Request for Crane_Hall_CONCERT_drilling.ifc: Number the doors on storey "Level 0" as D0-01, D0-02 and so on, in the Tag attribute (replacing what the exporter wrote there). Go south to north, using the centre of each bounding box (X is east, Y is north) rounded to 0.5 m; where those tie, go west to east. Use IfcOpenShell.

First a look at what the model holds.

```python
import ifcopenshell
import ifcopenshell.util.element
import ifcopenshell.util.placement

model = ifcopenshell.open("Crane_Hall_CONCERT_drilling.ifc")
print(model.schema)
storey = next(s for s in model.by_type("IfcBuildingStorey") if s.Name == "Level 0")
doors = [e for e in ifcopenshell.util.element.get_decomposition(storey) if e.is_a("IfcDoor")]
for e in sorted(doors, key=lambda e: e.id()):
    origin = ifcopenshell.util.placement.get_local_placement(e.ObjectPlacement)[:3, 3]
    print(e.id(), e.Tag, e.Name, origin.round(2) + 0.0, sep=" | ")
```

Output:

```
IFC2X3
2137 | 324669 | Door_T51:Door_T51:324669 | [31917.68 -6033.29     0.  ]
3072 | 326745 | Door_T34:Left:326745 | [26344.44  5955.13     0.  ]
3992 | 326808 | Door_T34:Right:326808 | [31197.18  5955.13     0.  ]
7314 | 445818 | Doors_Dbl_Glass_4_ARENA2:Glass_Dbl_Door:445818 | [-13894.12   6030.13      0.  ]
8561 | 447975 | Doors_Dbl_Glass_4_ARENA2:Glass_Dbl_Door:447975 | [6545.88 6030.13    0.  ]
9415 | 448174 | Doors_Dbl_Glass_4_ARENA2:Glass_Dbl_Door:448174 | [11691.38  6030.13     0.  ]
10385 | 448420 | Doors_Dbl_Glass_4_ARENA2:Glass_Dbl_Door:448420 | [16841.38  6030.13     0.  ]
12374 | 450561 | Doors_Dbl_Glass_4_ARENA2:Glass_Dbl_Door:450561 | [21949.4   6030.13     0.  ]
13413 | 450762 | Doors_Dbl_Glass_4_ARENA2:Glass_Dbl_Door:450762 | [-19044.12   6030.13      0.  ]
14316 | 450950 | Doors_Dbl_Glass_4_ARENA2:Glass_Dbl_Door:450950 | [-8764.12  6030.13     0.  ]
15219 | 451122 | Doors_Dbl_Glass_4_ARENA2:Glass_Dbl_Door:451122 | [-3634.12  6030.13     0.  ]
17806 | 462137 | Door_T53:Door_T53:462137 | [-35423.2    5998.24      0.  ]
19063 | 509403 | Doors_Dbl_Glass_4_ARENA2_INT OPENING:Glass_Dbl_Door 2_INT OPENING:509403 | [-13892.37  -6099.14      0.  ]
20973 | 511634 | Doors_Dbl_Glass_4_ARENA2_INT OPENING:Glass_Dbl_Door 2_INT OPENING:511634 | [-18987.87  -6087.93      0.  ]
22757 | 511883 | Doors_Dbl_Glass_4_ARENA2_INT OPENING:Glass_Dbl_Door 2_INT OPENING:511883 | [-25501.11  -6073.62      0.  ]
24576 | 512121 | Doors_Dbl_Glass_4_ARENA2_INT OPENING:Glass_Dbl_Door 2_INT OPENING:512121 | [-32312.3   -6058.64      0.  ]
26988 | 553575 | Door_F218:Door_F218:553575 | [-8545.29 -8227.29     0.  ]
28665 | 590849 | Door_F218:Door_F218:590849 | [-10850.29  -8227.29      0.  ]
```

```python
import ifcopenshell
import ifcopenshell.geom
import ifcopenshell.util.element
import ifcopenshell.util.shape

model = ifcopenshell.open("Crane_Hall_CONCERT_drilling.ifc")
settings = ifcopenshell.geom.settings()
settings.set("use-world-coords", True)


def centre(element):
    shape = ifcopenshell.geom.create_shape(settings, element)
    return ifcopenshell.util.shape.get_bbox_centroid(shape.geometry)


storey = next(s for s in model.by_type("IfcBuildingStorey") if s.Name == "Level 0")
doors = [e for e in ifcopenshell.util.element.get_decomposition(storey) if e.is_a("IfcDoor")]

# Insertion points can sit at a corner or the storey origin, so sort by the geometry (in metres).
centres = {e: centre(e) for e in doors}
doors.sort(key=lambda e: (round(centres[e][1] / 0.5), centres[e][0]))

for i, e in enumerate(doors, start=1):
    number = f"D0-{i:02d}"
    e.Tag = number
    print(e.id(), number)

model.write("Crane_Hall_CONCERT_drilling_updated.ifc")
```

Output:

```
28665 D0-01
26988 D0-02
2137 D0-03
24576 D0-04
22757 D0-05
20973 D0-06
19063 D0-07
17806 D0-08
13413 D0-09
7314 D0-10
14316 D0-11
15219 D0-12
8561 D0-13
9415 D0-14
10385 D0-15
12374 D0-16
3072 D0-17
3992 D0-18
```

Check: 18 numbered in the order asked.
